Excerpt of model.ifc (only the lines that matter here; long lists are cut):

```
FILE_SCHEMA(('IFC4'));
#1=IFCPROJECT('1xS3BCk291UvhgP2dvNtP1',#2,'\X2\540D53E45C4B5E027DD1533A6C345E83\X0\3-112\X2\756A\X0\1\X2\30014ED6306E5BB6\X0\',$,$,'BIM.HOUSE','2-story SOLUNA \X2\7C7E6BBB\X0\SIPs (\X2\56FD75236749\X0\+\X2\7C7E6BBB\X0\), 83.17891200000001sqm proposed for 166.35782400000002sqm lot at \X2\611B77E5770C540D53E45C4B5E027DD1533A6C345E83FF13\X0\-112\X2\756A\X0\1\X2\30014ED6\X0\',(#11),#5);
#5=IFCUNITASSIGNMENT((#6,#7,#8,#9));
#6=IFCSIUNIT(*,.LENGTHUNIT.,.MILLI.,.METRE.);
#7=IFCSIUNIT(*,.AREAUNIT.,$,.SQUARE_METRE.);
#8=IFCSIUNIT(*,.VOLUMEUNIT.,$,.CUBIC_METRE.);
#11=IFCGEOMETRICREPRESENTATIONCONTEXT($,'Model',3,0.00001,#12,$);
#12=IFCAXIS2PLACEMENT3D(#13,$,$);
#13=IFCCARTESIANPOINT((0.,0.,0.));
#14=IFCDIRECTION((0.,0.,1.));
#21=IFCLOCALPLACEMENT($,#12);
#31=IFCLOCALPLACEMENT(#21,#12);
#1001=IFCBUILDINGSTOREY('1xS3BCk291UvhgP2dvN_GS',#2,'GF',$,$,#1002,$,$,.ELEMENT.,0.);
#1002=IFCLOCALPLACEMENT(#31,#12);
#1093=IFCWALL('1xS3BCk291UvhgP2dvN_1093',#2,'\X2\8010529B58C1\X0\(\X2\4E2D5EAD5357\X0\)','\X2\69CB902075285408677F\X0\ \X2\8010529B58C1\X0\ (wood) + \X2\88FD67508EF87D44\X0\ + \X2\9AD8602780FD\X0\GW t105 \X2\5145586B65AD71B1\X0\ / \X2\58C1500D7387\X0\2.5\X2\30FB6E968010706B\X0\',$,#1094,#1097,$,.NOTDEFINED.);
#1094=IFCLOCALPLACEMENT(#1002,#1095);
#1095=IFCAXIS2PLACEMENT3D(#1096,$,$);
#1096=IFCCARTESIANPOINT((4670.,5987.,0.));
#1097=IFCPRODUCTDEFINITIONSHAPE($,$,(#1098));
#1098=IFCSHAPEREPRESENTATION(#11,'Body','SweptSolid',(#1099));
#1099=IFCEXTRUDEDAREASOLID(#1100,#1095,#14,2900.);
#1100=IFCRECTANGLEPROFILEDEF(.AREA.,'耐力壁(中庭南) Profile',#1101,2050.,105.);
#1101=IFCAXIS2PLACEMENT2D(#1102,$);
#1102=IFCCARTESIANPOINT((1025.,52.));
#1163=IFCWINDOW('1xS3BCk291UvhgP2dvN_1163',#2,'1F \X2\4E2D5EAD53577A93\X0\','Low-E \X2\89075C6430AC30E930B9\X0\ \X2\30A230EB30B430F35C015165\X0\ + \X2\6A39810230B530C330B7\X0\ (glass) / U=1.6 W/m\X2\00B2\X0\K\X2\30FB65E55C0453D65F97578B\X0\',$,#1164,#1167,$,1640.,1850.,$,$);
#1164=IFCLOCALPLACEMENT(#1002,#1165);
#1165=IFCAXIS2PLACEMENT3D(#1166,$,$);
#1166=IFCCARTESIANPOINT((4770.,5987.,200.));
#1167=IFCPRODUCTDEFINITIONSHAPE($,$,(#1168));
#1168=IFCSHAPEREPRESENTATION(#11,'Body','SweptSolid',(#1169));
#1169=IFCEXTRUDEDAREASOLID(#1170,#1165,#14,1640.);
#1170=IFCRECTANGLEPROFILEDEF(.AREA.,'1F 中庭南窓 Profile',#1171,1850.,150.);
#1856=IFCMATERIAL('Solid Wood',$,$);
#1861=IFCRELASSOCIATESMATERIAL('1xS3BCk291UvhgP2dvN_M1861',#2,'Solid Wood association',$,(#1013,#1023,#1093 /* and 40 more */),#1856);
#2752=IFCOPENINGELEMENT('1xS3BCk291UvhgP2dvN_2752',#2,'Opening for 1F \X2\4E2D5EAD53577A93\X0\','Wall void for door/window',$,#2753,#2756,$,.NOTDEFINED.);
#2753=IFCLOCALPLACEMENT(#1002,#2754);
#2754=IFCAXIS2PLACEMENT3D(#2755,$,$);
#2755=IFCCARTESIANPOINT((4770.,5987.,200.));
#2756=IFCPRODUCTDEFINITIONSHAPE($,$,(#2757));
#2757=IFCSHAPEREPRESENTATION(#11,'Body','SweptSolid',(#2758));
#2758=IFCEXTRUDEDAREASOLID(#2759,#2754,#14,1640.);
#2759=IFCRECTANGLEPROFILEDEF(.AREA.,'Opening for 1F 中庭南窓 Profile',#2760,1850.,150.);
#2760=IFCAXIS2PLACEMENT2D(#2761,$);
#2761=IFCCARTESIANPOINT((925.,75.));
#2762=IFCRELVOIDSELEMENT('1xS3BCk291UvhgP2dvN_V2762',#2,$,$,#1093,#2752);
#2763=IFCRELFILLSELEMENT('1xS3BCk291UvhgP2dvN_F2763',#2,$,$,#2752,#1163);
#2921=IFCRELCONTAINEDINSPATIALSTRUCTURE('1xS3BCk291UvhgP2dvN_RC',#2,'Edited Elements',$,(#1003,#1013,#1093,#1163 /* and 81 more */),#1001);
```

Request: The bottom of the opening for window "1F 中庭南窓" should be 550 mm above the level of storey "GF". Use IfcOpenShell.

```python
import numpy as np
import ifcopenshell
import ifcopenshell.api.geometry
import ifcopenshell.geom
import ifcopenshell.util.element
import ifcopenshell.util.placement
import ifcopenshell.util.shape
import ifcopenshell.util.unit

model = ifcopenshell.open("model.ifc")
unit_scale = ifcopenshell.util.unit.calculate_unit_scale(model)

window = model.by_guid("1xS3BCk291UvhgP2dvN_1163")
opening = window.FillsVoids[0].RelatingOpeningElement
storey = ifcopenshell.util.element.get_container(window, ifc_class="IfcBuildingStorey")
level = ifcopenshell.util.placement.get_local_placement(storey.ObjectPlacement)[2, 3]

# The opening's origin need not be at the sill, so measure its lowest point.
shape = ifcopenshell.geom.create_shape(ifcopenshell.geom.settings(), opening)
bottom = ifcopenshell.util.shape.get_shape_bottom_elevation(shape, shape.geometry) / unit_scale
dz = level + 550.0 - bottom

shift = np.array([0.0, 0.0, dz])
# The window is not placed relative to its opening, so move both.
for product in (opening, window):
    matrix = ifcopenshell.util.placement.get_local_placement(product.ObjectPlacement)
    matrix[:3, 3] += shift
    ifcopenshell.api.geometry.edit_object_placement(model, product=product, matrix=matrix, is_si=False)

print(f"moved by {dz * unit_scale:+.3f} m")

model.write("model_rev.ifc")
```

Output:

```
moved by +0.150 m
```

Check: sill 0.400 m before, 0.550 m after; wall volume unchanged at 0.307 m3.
